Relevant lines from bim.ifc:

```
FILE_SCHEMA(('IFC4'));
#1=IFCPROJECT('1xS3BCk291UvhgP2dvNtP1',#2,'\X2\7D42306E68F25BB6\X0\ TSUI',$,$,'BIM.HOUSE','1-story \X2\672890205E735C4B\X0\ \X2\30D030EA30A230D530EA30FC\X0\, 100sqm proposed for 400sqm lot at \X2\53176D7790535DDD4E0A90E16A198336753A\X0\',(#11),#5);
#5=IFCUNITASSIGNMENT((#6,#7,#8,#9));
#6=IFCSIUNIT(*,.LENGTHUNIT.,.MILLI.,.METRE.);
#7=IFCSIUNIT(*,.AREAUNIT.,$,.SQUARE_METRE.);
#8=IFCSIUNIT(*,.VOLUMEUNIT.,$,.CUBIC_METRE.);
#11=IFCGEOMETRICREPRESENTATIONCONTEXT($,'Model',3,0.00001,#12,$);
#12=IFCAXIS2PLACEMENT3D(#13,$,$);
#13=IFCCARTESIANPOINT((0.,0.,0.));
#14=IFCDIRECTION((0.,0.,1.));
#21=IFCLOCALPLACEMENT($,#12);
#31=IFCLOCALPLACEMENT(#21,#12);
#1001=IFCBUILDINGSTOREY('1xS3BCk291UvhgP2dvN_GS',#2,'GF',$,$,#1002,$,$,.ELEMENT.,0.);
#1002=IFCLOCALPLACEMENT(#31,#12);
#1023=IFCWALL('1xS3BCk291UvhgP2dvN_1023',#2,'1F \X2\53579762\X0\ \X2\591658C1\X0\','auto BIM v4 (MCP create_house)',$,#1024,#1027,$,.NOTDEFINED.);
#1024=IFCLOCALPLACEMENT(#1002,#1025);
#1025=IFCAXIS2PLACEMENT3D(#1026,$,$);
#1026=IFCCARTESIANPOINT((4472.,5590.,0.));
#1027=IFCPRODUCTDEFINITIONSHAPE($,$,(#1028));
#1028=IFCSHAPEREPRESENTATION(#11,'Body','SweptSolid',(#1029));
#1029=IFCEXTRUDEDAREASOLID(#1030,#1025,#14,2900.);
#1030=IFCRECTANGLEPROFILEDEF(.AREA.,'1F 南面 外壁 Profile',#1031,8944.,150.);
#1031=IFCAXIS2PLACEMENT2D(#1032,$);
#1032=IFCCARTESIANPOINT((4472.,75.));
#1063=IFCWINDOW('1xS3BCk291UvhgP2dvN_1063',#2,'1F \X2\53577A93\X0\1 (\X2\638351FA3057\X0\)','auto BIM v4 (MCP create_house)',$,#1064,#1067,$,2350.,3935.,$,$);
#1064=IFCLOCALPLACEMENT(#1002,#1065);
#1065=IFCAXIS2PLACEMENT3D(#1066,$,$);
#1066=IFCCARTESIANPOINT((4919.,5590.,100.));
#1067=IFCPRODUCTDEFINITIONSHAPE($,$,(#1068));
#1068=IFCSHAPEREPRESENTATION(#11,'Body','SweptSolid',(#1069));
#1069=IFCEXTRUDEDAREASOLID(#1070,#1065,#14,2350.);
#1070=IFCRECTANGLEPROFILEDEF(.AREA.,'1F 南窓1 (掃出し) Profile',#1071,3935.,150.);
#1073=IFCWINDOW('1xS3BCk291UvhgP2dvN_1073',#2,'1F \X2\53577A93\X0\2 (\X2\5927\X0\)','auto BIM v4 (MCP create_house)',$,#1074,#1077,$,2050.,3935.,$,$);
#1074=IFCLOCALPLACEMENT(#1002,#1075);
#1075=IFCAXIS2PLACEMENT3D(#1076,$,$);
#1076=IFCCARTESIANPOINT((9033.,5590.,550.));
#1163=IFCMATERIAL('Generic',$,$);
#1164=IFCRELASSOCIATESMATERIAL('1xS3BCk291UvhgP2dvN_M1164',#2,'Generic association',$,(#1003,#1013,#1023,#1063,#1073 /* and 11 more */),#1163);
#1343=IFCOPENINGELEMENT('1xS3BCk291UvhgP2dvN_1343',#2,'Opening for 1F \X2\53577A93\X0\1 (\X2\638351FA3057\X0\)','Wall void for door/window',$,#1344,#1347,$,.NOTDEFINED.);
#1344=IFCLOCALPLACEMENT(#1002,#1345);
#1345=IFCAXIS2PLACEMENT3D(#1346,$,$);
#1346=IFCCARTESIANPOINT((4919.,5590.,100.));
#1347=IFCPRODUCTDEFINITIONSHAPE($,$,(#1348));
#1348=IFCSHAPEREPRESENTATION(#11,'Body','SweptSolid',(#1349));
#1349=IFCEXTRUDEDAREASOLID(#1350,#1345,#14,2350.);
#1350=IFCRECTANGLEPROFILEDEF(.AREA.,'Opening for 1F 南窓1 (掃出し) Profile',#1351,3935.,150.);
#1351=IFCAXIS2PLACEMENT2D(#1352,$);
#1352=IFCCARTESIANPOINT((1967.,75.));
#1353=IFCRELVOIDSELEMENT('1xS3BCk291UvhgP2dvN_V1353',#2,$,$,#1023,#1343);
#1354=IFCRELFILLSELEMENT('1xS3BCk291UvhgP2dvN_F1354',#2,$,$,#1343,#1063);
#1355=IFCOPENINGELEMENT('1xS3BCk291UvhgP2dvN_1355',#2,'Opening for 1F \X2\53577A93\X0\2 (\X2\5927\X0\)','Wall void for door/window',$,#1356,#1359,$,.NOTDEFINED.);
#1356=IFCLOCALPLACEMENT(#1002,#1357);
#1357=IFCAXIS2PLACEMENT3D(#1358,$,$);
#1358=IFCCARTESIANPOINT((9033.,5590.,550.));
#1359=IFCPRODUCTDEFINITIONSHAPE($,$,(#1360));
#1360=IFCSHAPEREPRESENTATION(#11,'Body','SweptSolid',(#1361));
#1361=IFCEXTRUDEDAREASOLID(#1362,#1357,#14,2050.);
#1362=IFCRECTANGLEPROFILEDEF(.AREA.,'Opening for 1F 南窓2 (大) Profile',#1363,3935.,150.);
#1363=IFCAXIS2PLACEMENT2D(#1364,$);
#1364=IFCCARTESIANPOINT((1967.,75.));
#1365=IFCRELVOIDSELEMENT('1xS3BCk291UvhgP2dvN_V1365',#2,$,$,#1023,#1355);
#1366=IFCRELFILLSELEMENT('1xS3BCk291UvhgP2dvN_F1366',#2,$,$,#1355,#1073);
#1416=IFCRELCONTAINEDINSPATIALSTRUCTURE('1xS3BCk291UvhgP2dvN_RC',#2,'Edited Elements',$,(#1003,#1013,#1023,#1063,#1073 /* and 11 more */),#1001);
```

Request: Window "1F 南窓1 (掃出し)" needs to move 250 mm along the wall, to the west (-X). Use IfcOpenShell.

```python
import ifcopenshell
import ifcopenshell.api.geometry
import ifcopenshell.util.placement
import ifcopenshell.util.unit

model = ifcopenshell.open("bim.ifc")
unit_scale = ifcopenshell.util.unit.calculate_unit_scale(model)

window = model.by_guid("1xS3BCk291UvhgP2dvN_1063")
opening = window.FillsVoids[0].RelatingOpeningElement
wall = opening.VoidsElements[0].RelatingBuildingElement

wall_matrix = ifcopenshell.util.placement.get_local_placement(wall.ObjectPlacement)
shift = wall_matrix[:3, 0] * -0.25 / unit_scale
before = ifcopenshell.util.placement.get_local_placement(window.ObjectPlacement)[:3, 3].copy()

# The window is not placed relative to its opening, so move both.
for product in (opening, window):
    matrix = ifcopenshell.util.placement.get_local_placement(product.ObjectPlacement)
    matrix[:3, 3] += shift
    ifcopenshell.api.geometry.edit_object_placement(model, product=product, matrix=matrix, is_si=False)

after = ifcopenshell.util.placement.get_local_placement(window.ObjectPlacement)[:3, 3]
print("window moved by", (after - before).round(3) + 0.0)

model.write("bim_rev.ifc")
```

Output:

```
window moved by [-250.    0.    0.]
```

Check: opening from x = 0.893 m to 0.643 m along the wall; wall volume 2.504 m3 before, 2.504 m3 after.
